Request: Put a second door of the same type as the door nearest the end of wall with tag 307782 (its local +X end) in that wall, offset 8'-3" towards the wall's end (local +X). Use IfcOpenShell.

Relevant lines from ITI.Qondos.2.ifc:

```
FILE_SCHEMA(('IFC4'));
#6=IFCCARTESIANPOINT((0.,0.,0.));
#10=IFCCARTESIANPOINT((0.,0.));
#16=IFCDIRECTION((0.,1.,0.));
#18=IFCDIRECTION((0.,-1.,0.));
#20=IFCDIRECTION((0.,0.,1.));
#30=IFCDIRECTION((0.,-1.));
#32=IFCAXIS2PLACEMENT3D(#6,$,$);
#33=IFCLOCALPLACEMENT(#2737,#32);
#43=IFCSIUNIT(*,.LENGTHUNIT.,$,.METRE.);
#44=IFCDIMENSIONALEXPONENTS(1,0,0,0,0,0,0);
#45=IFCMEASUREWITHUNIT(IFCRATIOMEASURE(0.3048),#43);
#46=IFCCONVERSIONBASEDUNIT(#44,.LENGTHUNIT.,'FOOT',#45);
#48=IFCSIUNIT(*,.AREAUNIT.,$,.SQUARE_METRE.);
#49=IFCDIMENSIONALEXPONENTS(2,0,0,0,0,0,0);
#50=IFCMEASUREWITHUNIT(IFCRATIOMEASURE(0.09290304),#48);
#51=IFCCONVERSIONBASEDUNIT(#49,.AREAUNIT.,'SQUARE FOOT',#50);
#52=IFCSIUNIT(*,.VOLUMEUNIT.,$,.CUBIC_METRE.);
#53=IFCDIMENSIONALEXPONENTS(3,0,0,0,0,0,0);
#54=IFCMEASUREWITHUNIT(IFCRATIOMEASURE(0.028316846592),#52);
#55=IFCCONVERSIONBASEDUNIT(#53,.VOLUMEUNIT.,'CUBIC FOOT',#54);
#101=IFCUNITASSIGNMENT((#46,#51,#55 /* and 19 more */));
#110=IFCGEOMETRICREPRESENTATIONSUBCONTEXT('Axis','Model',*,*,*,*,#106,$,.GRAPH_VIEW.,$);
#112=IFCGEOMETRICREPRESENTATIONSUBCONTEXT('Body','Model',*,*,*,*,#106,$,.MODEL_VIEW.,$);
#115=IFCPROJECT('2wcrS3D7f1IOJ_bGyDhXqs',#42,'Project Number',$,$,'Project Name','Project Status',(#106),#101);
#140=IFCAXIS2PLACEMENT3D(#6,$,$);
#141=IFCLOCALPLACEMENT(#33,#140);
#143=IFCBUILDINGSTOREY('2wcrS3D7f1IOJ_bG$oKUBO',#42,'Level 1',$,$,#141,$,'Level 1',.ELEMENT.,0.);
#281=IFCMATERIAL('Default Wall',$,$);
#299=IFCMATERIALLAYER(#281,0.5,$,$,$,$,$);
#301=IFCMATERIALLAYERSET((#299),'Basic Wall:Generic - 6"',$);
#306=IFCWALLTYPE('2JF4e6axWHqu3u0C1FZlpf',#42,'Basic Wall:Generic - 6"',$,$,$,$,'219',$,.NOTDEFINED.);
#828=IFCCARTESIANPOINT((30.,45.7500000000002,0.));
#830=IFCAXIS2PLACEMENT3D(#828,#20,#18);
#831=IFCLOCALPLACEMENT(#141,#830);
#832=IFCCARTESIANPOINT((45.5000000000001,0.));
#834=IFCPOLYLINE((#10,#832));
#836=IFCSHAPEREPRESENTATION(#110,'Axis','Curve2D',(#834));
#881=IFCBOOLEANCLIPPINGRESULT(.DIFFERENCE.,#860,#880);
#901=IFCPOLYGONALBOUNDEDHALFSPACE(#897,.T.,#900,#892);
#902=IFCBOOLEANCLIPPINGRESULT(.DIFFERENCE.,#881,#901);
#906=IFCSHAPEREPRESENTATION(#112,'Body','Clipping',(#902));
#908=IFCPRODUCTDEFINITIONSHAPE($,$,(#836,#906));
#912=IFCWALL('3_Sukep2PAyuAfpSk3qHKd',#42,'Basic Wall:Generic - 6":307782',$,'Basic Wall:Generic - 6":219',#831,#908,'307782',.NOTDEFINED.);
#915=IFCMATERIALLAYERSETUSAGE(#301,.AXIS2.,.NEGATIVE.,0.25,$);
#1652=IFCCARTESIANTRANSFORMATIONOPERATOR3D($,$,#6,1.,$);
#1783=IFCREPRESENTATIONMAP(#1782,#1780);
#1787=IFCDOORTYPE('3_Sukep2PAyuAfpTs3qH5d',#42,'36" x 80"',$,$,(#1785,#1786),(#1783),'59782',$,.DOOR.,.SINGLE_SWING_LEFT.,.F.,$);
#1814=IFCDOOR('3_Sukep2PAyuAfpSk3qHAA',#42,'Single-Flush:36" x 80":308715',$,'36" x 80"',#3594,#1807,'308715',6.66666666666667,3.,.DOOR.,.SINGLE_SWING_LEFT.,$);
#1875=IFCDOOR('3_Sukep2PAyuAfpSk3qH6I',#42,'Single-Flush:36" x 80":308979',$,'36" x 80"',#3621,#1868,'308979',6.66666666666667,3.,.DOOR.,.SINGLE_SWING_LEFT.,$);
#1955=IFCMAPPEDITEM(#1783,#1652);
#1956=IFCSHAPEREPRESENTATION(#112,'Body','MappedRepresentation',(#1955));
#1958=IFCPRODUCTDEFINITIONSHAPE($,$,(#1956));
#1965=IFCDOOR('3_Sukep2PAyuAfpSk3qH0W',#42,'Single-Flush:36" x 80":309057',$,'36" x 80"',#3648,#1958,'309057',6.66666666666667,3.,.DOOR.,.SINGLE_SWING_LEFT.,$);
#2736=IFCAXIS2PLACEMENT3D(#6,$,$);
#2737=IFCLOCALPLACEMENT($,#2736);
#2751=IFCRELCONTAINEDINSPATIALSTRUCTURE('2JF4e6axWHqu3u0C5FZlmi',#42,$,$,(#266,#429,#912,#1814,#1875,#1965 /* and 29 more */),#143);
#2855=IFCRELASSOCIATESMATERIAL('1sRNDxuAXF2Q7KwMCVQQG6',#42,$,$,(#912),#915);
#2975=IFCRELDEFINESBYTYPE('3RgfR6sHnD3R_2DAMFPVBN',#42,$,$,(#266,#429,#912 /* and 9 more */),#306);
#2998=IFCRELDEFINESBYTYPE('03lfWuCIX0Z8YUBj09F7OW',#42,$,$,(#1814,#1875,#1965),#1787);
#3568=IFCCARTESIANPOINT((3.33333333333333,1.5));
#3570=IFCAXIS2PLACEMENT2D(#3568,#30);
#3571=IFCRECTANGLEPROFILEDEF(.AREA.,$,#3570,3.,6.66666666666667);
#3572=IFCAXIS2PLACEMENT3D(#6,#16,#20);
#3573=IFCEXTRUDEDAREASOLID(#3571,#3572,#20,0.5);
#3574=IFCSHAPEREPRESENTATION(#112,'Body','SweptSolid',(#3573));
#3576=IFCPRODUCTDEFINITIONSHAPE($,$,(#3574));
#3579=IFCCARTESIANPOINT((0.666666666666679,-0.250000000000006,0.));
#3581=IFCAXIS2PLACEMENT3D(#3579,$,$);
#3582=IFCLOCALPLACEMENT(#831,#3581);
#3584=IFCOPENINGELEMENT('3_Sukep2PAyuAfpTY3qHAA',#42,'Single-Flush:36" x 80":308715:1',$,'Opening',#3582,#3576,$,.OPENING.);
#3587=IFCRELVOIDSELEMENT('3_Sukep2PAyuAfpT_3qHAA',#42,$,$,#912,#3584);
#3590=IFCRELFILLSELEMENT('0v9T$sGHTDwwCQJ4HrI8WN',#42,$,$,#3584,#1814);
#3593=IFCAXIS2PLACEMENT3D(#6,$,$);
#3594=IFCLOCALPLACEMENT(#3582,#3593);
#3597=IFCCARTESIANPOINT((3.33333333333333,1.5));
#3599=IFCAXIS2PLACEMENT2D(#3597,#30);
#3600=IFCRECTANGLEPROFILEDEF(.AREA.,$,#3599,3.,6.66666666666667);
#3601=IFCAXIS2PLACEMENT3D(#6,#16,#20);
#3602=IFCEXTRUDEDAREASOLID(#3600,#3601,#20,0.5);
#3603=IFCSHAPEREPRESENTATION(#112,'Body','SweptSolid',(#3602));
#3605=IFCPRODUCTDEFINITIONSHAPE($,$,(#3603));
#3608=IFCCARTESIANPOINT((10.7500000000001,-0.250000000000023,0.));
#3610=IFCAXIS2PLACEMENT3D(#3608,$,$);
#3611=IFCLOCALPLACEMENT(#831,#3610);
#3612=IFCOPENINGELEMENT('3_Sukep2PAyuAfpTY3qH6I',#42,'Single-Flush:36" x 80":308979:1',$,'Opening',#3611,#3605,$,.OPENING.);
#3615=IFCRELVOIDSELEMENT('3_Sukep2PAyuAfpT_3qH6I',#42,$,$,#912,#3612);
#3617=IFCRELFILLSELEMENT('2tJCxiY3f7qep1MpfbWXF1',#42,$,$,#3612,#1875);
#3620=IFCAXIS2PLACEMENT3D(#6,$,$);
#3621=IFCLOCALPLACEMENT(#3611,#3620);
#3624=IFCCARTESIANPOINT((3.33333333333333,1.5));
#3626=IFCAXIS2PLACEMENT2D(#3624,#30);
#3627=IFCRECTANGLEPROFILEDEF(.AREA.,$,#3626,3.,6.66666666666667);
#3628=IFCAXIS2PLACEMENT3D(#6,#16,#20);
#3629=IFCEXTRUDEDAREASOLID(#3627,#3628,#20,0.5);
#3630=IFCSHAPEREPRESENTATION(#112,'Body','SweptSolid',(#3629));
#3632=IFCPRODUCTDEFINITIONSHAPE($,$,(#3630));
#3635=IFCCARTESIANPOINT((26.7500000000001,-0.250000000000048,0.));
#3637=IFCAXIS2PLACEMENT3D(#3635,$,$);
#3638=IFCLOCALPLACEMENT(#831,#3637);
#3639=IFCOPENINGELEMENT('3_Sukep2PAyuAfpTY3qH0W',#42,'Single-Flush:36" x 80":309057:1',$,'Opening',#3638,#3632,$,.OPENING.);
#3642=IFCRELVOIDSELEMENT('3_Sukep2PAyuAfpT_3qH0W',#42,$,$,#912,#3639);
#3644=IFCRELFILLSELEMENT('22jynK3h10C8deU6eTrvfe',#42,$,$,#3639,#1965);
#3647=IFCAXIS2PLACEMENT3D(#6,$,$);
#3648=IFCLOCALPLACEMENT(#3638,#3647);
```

```python
import ifcopenshell
import ifcopenshell.api.feature
import ifcopenshell.api.geometry
import ifcopenshell.api.root
import ifcopenshell.geom
import ifcopenshell.util.element
import ifcopenshell.util.placement
import ifcopenshell.util.shape
import ifcopenshell.util.unit

model = ifcopenshell.open("ITI.Qondos.2.ifc")
unit_scale = ifcopenshell.util.unit.calculate_unit_scale(model)
settings = ifcopenshell.geom.settings()


def volume(element):
    """Net volume in cubic metres, openings subtracted."""
    shape = ifcopenshell.geom.create_shape(settings, element)
    return ifcopenshell.util.shape.get_volume(shape.geometry)


def reuse_history(source, copy):
    """copy_class also copies each property set's owner history, people and application; keep the originals."""
    for rel in copy.IsDefinedBy:
        if rel.is_a("IfcRelDefinesByProperties") and (history := rel.RelatingPropertyDefinition.OwnerHistory):
            rel.RelatingPropertyDefinition.OwnerHistory = source.OwnerHistory
            ifcopenshell.util.element.remove_deep2(model, history)


door = model.by_guid("3_Sukep2PAyuAfpSk3qH0W")
opening = door.FillsVoids[0].RelatingOpeningElement
wall = opening.VoidsElements[0].RelatingBuildingElement
before = volume(wall)
shift = ifcopenshell.util.placement.get_local_placement(wall.ObjectPlacement)[:3, 0] * 99 * 0.0254 / unit_scale

# copy_class copies the void relationship, type, container and properties, but no geometry.
new_opening = ifcopenshell.api.root.copy_class(model, product=opening)
new_opening.Representation = ifcopenshell.util.element.copy_deep(
    model, opening.Representation, exclude=["IfcGeometricRepresentationContext", "IfcRepresentationMap"]
)
new_opening.Name = 'Single-Flush:36" x 80"'
new_door = ifcopenshell.api.root.copy_class(model, product=door)
new_door.Representation = ifcopenshell.util.element.copy_deep(
    model, door.Representation, exclude=["IfcGeometricRepresentationContext", "IfcRepresentationMap"]
)
new_door.Name = 'Single-Flush:36" x 80"'
new_door.Tag = None
reuse_history(door, new_door)
ifcopenshell.api.feature.add_filling(model, opening=new_opening, element=new_door)

for old, new in ((opening, new_opening), (door, new_door)):
    matrix = ifcopenshell.util.placement.get_local_placement(old.ObjectPlacement)
    matrix[:3, 3] += shift
    ifcopenshell.api.geometry.edit_object_placement(model, product=new, matrix=matrix, is_si=False)

after = volume(wall)

print(f"wall volume {before:.3f} -> {after:.3f} m3")

model.write("ITI.Qondos.2-out.ifc")
```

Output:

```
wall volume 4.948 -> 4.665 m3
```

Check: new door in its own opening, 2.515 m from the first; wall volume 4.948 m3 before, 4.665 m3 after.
